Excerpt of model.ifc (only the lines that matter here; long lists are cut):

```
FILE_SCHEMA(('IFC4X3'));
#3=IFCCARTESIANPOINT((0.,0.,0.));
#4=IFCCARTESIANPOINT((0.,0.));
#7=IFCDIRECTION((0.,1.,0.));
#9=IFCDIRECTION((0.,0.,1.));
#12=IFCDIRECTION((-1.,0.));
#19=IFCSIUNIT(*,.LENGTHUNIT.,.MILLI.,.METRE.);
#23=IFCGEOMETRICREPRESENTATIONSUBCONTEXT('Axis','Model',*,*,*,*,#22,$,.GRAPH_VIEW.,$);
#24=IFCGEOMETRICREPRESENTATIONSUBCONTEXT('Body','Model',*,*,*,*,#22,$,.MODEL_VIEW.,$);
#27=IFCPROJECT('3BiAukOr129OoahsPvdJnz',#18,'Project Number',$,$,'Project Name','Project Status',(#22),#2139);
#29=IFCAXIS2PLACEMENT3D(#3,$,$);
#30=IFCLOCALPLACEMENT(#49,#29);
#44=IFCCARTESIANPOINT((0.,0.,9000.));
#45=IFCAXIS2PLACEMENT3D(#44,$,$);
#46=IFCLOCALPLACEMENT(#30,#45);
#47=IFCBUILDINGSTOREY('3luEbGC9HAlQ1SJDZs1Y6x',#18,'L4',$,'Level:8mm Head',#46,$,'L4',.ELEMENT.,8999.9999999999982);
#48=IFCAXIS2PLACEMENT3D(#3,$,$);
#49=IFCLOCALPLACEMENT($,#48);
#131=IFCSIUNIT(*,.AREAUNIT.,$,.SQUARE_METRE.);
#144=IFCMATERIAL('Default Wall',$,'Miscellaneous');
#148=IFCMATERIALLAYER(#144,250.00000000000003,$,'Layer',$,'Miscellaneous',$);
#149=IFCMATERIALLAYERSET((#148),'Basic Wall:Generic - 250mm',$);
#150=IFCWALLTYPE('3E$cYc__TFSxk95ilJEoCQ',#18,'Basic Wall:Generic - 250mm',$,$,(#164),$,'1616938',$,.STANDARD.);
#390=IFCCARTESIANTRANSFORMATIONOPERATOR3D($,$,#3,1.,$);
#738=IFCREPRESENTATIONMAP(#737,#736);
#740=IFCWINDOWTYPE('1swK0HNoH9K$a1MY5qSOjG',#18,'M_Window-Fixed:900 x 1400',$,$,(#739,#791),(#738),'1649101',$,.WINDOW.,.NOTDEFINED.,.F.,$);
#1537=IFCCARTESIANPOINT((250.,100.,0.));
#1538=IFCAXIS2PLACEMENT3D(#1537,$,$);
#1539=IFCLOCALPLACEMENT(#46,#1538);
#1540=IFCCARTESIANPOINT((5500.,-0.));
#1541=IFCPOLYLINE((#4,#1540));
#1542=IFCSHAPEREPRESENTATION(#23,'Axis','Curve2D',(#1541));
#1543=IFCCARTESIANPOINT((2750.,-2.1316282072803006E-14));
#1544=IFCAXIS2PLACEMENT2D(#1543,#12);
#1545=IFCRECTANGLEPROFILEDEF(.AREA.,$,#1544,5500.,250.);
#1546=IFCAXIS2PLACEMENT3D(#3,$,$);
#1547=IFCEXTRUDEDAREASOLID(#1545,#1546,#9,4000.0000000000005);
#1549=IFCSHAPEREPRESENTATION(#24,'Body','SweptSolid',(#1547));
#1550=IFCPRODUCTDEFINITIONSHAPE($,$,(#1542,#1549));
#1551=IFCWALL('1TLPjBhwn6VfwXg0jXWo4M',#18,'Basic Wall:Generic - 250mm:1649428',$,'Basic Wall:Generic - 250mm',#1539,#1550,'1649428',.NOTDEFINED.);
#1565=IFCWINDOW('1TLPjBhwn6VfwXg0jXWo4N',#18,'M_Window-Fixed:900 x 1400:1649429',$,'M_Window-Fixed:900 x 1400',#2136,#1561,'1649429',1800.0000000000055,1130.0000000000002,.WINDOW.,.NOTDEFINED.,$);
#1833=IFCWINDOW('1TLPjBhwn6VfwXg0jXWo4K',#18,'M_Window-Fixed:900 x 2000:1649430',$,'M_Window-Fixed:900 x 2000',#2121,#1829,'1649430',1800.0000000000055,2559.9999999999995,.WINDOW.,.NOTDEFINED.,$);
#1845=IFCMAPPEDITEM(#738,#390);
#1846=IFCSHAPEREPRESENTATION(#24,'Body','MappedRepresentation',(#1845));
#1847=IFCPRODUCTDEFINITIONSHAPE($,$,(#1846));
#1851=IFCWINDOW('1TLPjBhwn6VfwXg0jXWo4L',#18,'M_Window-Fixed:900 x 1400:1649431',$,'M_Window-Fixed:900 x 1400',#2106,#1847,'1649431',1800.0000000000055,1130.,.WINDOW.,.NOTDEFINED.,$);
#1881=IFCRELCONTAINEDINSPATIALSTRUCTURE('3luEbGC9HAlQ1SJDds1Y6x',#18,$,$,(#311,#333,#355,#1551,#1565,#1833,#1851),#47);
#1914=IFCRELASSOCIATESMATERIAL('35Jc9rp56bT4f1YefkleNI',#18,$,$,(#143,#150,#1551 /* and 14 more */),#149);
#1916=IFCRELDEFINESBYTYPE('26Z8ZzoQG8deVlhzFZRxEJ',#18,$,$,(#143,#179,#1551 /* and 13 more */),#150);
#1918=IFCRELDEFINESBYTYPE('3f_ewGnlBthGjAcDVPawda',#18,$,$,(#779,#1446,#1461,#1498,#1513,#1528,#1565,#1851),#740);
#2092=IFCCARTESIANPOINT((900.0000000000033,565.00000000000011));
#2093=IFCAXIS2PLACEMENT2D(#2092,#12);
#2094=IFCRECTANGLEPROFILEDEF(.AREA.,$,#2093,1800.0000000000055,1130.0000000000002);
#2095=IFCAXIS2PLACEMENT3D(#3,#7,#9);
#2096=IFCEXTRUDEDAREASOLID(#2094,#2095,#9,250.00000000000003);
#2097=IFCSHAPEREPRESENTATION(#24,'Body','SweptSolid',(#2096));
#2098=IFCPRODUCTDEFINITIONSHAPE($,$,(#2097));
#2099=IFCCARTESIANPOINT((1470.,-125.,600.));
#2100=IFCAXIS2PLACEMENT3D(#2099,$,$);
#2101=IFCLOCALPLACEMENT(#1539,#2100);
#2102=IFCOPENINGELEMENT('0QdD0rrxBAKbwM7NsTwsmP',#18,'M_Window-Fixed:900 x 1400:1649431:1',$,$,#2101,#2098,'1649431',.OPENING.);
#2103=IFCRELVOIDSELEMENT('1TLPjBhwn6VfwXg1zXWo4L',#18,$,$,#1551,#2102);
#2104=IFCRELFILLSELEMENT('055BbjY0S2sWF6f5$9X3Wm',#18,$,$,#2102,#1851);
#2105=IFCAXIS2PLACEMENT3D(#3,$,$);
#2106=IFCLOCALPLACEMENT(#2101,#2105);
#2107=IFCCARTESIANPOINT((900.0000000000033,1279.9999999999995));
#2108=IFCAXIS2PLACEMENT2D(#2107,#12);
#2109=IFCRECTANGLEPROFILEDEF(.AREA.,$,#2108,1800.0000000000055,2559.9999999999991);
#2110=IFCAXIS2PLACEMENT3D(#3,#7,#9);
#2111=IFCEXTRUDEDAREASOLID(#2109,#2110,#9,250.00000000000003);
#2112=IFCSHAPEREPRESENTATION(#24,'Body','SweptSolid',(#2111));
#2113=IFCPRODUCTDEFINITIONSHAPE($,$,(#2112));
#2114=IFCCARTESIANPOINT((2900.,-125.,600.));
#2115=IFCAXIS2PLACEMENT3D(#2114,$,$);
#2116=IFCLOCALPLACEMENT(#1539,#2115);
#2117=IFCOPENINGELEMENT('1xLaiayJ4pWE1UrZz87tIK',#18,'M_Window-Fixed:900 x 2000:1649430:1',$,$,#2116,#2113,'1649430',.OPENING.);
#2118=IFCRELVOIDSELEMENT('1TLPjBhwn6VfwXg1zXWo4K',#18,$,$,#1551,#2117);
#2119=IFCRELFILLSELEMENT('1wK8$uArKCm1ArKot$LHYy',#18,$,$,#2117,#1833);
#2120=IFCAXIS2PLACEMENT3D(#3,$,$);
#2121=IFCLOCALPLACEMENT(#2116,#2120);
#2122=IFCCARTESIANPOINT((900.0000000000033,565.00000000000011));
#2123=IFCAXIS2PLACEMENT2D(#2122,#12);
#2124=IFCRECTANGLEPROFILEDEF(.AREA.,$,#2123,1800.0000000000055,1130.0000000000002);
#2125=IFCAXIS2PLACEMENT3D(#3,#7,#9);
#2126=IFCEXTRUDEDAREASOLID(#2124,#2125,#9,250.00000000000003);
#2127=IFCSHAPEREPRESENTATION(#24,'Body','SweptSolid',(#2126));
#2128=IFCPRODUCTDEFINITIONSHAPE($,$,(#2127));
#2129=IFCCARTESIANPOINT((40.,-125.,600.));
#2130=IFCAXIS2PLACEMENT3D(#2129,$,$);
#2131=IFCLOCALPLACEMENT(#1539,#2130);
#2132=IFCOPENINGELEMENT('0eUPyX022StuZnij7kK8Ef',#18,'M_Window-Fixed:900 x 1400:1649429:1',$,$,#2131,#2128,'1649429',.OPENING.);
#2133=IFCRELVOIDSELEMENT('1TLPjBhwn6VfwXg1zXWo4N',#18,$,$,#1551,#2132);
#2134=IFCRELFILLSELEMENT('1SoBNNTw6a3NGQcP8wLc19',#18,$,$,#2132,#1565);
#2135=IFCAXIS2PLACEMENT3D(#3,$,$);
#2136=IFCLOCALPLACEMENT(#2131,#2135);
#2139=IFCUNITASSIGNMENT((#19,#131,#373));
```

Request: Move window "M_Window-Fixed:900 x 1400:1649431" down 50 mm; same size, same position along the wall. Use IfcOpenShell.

```python
import numpy as np
import ifcopenshell
import ifcopenshell.api.geometry
import ifcopenshell.util.placement
import ifcopenshell.util.unit

model = ifcopenshell.open("model.ifc")
unit_scale = ifcopenshell.util.unit.calculate_unit_scale(model)

window = model.by_guid("1TLPjBhwn6VfwXg0jXWo4L")
opening = window.FillsVoids[0].RelatingOpeningElement
dz = -0.05 / unit_scale

shift = np.array([0.0, 0.0, dz])
# The window is placed relative to its opening, so it follows when the opening moves.
matrix = ifcopenshell.util.placement.get_local_placement(opening.ObjectPlacement)
matrix[:3, 3] += shift
ifcopenshell.api.geometry.edit_object_placement(
    model, product=opening, matrix=matrix, is_si=False, should_transform_children=True
)

print(f"moved by {dz * unit_scale:+.3f} m")

model.write("model-out.ifc")
```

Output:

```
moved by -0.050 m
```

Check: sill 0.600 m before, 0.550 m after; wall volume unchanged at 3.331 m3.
